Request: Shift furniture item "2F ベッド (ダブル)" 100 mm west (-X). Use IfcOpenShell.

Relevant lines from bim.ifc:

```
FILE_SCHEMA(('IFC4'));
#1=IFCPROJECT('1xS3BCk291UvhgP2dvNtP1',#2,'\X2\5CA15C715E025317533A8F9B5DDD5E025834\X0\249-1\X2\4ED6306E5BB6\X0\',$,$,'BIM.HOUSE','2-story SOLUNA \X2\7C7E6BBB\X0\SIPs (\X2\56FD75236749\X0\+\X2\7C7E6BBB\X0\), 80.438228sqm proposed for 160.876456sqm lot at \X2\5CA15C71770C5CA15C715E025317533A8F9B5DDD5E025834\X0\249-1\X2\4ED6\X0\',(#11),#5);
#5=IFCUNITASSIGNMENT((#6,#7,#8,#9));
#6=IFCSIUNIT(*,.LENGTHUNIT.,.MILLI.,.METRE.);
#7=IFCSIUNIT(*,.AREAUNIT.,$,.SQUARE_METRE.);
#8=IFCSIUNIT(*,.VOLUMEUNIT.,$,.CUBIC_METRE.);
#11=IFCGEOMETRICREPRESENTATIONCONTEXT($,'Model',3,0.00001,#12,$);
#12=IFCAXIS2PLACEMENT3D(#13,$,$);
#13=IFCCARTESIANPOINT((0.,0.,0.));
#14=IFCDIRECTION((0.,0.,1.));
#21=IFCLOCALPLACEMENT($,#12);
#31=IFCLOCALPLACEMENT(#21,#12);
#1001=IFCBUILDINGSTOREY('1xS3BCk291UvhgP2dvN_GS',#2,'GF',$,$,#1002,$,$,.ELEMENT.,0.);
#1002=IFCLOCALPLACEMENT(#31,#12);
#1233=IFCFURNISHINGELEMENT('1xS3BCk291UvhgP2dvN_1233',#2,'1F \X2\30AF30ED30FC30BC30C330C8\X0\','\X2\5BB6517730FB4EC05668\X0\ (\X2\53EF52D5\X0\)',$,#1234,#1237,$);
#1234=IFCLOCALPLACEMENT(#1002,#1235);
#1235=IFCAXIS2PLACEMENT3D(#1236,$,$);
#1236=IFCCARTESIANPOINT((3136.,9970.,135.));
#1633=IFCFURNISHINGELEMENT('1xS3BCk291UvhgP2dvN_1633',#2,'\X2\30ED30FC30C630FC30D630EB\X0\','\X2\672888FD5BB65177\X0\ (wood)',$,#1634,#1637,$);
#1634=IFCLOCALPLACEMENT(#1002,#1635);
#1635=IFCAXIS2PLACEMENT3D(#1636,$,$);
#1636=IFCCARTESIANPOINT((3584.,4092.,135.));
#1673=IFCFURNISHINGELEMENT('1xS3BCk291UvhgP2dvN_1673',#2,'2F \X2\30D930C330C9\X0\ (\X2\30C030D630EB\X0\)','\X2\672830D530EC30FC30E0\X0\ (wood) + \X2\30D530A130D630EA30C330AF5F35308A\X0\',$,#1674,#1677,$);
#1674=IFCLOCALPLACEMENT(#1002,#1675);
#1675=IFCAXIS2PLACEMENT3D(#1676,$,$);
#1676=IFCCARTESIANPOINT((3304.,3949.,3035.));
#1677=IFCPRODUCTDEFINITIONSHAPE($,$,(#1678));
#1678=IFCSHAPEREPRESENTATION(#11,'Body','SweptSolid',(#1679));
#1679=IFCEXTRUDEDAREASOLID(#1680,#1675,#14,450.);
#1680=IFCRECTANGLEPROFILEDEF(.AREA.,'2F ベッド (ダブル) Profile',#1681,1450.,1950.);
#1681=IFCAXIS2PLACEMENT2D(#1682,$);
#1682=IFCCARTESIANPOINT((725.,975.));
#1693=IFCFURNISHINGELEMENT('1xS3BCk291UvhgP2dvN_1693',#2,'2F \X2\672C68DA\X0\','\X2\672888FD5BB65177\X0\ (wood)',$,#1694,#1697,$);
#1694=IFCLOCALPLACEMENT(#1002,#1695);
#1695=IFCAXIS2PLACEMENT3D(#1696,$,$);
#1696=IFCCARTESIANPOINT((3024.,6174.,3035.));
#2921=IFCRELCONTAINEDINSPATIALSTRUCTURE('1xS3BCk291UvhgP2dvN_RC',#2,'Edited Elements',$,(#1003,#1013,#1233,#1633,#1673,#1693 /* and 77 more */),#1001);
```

```python
import ifcopenshell
import ifcopenshell.api.geometry
import ifcopenshell.util.placement
import ifcopenshell.util.unit

model = ifcopenshell.open("bim.ifc")
unit_scale = ifcopenshell.util.unit.calculate_unit_scale(model)

item = model.by_id(1673)
matrix = ifcopenshell.util.placement.get_local_placement(item.ObjectPlacement)
matrix[0, 3] -= 0.1 / unit_scale
ifcopenshell.api.geometry.edit_object_placement(model, product=item, matrix=matrix, is_si=False)

print(ifcopenshell.util.placement.get_local_placement(item.ObjectPlacement).round(3) + 0.0)

model.write("bim_edited.ifc")
```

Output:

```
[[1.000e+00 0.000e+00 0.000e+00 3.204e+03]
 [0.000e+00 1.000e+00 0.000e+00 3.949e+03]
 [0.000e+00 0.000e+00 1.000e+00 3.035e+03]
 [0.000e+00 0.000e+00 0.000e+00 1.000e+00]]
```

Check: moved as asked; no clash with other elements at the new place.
